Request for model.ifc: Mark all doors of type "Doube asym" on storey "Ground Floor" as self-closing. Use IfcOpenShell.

First a look at what the model holds.

```python
import ifcopenshell
import ifcopenshell.util.element

model = ifcopenshell.open("model.ifc")
print(model.schema)
storey = next(s for s in model.by_type("IfcBuildingStorey") if s.Name == "Ground Floor")
doors = [e for e in ifcopenshell.util.element.get_decomposition(storey) if e.is_a("IfcDoor")]
seen = {}
for e in doors:
    element_type = ifcopenshell.util.element.get_type(e)
    key = (element_type.Name if element_type != e and element_type else None, ifcopenshell.util.element.get_pset(e, "Pset_DoorCommon", "SelfClosing"))
    seen[key] = seen.get(key, 0) + 1
for (name, value), count in sorted(seen.items(), key=str):
    print(count, "x", name, "|", value)
```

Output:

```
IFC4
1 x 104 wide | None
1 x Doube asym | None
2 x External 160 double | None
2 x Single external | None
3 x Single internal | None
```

```python
import ifcopenshell
import ifcopenshell.api.pset
import ifcopenshell.util.element

model = ifcopenshell.open("model.ifc")

storey = next(s for s in model.by_type("IfcBuildingStorey") if s.Name == "Ground Floor")
doors = [e for e in ifcopenshell.util.element.get_decomposition(storey) if e.is_a("IfcDoor")]

count = 0
for e in doors:
    element_type = ifcopenshell.util.element.get_type(e)
    if element_type in (None, e) or element_type.Name != "Doube asym":
        continue
    # add_pset returns the element's existing set when there is one.
    pset = ifcopenshell.api.pset.add_pset(model, product=e, name="Pset_DoorCommon")
    ifcopenshell.api.pset.edit_pset(model, pset=pset, properties={"SelfClosing": True})
    count += 1

print(count, "doors updated")

model.write("model-out.ifc")
```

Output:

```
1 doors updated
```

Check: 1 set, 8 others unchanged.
